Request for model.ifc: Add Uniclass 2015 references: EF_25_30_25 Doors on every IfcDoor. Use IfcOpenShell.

First a look at what the model holds.

```python
import ifcopenshell

model = ifcopenshell.open("model.ifc")
print(model.schema)
print("classifications:", [c.Name for c in model.by_type("IfcClassification")])
for ifc_class in ("IfcDoor", "IfcRoof", "IfcStair", "IfcWall", "IfcWindow"):
    print(ifc_class, len(model.by_type(ifc_class)))
```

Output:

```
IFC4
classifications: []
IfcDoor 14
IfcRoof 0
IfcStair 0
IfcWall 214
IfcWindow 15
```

```python
import ifcopenshell
import ifcopenshell.api.classification

model = ifcopenshell.open("model.ifc")

system = ifcopenshell.api.classification.add_classification(model, classification="Uniclass 2015")

codes = {
    "IfcDoor": ("EF_25_30_25", "Doors"),
}
for ifc_class, (code, name) in codes.items():
    products = model.by_type(ifc_class)
    ifcopenshell.api.classification.add_reference(
        model, products=products, classification=system, identification=code, name=name
    )
    print(code, len(products))

model.write("model_updated.ifc")
```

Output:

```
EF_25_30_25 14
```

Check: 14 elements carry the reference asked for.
